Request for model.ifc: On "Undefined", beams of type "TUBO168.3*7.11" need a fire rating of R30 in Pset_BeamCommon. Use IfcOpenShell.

First a look at what the model holds.

```python
import ifcopenshell
import ifcopenshell.util.element

model = ifcopenshell.open("model.ifc")
print(model.schema)
storey = next(s for s in model.by_type("IfcBuildingStorey") if s.Name == "Undefined")
beams = [e for e in ifcopenshell.util.element.get_decomposition(storey) if e.is_a("IfcBeam")]
seen = {}
for e in beams:
    element_type = ifcopenshell.util.element.get_type(e)
    key = (element_type.Name if element_type != e and element_type else None, ifcopenshell.util.element.get_pset(e, "Pset_BeamCommon", "FireRating"))
    seen[key] = seen.get(key, 0) + 1
for (name, value), count in sorted(seen.items(), key=str):
    print(count, "x", name, "|", value)
```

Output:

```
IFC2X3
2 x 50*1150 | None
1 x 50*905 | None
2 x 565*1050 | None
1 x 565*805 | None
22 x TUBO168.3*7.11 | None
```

```python
import ifcopenshell
import ifcopenshell.api.pset
import ifcopenshell.util.element

model = ifcopenshell.open("model.ifc")

storey = next(s for s in model.by_type("IfcBuildingStorey") if s.Name == "Undefined")
beams = [e for e in ifcopenshell.util.element.get_decomposition(storey) if e.is_a("IfcBeam")]

count = 0
for e in beams:
    element_type = ifcopenshell.util.element.get_type(e)
    if element_type in (None, e) or element_type.Name != "TUBO168.3*7.11":
        continue
    found = ifcopenshell.util.element.get_pset(e, "Pset_BeamCommon", should_inherit=False)
    if found:
        pset = model.by_id(found["id"])
        if len(ifcopenshell.util.element.get_elements_by_pset(pset)) > 1:
            pset = ifcopenshell.api.pset.unshare_pset(model, products=[e], pset=pset)[0]
    else:
        pset = ifcopenshell.api.pset.add_pset(model, product=e, name="Pset_BeamCommon")
    ifcopenshell.api.pset.edit_pset(model, pset=pset, properties={"FireRating": "R30"})
    count += 1

print(count, "beams updated")

model.write("model-out.ifc")
```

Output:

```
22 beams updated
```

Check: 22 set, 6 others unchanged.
